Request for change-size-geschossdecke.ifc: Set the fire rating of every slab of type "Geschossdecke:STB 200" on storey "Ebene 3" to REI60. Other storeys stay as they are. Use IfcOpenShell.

First a look at what the model holds.

```python
import ifcopenshell
import ifcopenshell.util.element

model = ifcopenshell.open("change-size-geschossdecke.ifc")
print(model.schema)
storey = next(s for s in model.by_type("IfcBuildingStorey") if s.Name == "Ebene 3")
slabs = [e for e in ifcopenshell.util.element.get_decomposition(storey) if e.is_a("IfcSlab")]
seen = {}
for e in slabs:
    element_type = ifcopenshell.util.element.get_type(e)
    key = (element_type.Name if element_type != e and element_type else None, ifcopenshell.util.element.get_pset(e, "Pset_SlabCommon", "FireRating"))
    seen[key] = seen.get(key, 0) + 1
for (name, value), count in sorted(seen.items(), key=str):
    print(count, "x", name, "|", value)
```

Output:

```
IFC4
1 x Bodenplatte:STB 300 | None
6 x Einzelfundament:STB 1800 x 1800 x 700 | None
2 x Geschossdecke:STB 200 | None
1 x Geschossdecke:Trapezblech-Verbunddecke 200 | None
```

```python
import ifcopenshell
import ifcopenshell.api.pset
import ifcopenshell.util.element

model = ifcopenshell.open("change-size-geschossdecke.ifc")

storey = next(s for s in model.by_type("IfcBuildingStorey") if s.Name == "Ebene 3")
slabs = [e for e in ifcopenshell.util.element.get_decomposition(storey) if e.is_a("IfcSlab")]

count = 0
for e in slabs:
    element_type = ifcopenshell.util.element.get_type(e)
    if element_type in (None, e) or element_type.Name != "Geschossdecke:STB 200":
        continue
    # add_pset returns the element's existing set when there is one.
    pset = ifcopenshell.api.pset.add_pset(model, product=e, name="Pset_SlabCommon")
    ifcopenshell.api.pset.edit_pset(model, pset=pset, properties={"FireRating": "REI60"})
    count += 1

print(count, "slabs updated")

model.write("change-size-geschossdecke_rev.ifc")
```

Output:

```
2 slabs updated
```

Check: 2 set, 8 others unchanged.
